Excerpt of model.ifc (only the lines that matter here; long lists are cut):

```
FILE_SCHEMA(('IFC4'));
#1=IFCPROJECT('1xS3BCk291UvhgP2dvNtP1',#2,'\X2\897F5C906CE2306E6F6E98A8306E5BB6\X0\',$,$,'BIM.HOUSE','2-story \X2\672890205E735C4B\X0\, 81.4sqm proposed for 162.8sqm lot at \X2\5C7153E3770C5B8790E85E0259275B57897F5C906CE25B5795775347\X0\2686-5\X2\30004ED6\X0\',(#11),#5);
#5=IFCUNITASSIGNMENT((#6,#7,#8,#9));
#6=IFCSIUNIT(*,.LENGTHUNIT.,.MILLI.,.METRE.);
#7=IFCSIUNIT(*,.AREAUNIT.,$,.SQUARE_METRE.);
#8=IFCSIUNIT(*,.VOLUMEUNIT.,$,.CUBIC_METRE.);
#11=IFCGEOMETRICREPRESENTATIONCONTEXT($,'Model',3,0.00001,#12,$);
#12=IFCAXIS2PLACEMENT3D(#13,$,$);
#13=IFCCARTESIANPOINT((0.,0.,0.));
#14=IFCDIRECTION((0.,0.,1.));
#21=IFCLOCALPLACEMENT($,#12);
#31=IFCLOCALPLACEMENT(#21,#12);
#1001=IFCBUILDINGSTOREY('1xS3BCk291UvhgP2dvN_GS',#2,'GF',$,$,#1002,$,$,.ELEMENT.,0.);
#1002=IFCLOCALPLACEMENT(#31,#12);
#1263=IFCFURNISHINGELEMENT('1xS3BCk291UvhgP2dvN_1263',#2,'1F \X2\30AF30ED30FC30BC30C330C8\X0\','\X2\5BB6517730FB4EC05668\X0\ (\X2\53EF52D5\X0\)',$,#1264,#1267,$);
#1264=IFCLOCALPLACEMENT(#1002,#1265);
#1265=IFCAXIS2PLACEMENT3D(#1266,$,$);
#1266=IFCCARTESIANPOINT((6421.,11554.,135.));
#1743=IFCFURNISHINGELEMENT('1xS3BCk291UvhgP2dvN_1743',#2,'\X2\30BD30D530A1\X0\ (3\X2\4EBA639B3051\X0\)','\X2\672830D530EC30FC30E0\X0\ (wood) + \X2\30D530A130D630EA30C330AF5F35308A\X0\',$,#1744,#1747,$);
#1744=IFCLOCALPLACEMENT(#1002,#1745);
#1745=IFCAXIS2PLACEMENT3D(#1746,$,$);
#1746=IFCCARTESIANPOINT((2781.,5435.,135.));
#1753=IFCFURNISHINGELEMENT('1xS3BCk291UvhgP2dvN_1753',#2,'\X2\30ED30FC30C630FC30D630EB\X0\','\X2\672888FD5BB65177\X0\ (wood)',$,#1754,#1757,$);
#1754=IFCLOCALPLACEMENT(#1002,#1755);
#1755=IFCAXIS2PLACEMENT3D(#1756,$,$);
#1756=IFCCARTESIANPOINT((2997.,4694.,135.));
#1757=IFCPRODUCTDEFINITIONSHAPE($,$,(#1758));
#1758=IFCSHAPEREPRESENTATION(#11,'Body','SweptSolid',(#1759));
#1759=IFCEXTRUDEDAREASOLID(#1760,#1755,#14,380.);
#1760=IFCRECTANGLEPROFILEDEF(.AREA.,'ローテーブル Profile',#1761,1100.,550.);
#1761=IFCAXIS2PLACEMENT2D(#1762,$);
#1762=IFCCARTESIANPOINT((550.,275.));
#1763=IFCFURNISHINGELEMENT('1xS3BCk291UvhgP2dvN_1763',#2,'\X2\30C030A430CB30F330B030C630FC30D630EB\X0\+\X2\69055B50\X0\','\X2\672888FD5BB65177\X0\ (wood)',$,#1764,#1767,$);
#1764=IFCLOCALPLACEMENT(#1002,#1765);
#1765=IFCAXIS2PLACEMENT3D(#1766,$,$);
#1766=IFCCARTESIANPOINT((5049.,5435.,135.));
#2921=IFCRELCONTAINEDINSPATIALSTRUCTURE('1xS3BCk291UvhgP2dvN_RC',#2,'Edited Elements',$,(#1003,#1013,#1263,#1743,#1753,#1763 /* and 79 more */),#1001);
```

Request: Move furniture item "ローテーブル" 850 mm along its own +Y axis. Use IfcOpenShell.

```python
import ifcopenshell
import ifcopenshell.api.geometry
import ifcopenshell.util.placement

model = ifcopenshell.open("model.ifc")

item = model.by_id(1753)
matrix = ifcopenshell.util.placement.get_local_placement(item.ObjectPlacement)
matrix[:3, 3] += matrix[:3, 1] * 850.0
ifcopenshell.api.geometry.edit_object_placement(model, product=item, matrix=matrix, is_si=False)

print(ifcopenshell.util.placement.get_local_placement(item.ObjectPlacement).round(3) + 0.0)

model.write("model_v2.ifc")
```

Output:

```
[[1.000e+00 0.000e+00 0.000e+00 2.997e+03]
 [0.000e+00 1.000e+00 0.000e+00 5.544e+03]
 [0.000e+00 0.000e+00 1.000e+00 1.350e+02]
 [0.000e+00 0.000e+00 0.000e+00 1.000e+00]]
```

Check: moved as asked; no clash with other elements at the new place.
